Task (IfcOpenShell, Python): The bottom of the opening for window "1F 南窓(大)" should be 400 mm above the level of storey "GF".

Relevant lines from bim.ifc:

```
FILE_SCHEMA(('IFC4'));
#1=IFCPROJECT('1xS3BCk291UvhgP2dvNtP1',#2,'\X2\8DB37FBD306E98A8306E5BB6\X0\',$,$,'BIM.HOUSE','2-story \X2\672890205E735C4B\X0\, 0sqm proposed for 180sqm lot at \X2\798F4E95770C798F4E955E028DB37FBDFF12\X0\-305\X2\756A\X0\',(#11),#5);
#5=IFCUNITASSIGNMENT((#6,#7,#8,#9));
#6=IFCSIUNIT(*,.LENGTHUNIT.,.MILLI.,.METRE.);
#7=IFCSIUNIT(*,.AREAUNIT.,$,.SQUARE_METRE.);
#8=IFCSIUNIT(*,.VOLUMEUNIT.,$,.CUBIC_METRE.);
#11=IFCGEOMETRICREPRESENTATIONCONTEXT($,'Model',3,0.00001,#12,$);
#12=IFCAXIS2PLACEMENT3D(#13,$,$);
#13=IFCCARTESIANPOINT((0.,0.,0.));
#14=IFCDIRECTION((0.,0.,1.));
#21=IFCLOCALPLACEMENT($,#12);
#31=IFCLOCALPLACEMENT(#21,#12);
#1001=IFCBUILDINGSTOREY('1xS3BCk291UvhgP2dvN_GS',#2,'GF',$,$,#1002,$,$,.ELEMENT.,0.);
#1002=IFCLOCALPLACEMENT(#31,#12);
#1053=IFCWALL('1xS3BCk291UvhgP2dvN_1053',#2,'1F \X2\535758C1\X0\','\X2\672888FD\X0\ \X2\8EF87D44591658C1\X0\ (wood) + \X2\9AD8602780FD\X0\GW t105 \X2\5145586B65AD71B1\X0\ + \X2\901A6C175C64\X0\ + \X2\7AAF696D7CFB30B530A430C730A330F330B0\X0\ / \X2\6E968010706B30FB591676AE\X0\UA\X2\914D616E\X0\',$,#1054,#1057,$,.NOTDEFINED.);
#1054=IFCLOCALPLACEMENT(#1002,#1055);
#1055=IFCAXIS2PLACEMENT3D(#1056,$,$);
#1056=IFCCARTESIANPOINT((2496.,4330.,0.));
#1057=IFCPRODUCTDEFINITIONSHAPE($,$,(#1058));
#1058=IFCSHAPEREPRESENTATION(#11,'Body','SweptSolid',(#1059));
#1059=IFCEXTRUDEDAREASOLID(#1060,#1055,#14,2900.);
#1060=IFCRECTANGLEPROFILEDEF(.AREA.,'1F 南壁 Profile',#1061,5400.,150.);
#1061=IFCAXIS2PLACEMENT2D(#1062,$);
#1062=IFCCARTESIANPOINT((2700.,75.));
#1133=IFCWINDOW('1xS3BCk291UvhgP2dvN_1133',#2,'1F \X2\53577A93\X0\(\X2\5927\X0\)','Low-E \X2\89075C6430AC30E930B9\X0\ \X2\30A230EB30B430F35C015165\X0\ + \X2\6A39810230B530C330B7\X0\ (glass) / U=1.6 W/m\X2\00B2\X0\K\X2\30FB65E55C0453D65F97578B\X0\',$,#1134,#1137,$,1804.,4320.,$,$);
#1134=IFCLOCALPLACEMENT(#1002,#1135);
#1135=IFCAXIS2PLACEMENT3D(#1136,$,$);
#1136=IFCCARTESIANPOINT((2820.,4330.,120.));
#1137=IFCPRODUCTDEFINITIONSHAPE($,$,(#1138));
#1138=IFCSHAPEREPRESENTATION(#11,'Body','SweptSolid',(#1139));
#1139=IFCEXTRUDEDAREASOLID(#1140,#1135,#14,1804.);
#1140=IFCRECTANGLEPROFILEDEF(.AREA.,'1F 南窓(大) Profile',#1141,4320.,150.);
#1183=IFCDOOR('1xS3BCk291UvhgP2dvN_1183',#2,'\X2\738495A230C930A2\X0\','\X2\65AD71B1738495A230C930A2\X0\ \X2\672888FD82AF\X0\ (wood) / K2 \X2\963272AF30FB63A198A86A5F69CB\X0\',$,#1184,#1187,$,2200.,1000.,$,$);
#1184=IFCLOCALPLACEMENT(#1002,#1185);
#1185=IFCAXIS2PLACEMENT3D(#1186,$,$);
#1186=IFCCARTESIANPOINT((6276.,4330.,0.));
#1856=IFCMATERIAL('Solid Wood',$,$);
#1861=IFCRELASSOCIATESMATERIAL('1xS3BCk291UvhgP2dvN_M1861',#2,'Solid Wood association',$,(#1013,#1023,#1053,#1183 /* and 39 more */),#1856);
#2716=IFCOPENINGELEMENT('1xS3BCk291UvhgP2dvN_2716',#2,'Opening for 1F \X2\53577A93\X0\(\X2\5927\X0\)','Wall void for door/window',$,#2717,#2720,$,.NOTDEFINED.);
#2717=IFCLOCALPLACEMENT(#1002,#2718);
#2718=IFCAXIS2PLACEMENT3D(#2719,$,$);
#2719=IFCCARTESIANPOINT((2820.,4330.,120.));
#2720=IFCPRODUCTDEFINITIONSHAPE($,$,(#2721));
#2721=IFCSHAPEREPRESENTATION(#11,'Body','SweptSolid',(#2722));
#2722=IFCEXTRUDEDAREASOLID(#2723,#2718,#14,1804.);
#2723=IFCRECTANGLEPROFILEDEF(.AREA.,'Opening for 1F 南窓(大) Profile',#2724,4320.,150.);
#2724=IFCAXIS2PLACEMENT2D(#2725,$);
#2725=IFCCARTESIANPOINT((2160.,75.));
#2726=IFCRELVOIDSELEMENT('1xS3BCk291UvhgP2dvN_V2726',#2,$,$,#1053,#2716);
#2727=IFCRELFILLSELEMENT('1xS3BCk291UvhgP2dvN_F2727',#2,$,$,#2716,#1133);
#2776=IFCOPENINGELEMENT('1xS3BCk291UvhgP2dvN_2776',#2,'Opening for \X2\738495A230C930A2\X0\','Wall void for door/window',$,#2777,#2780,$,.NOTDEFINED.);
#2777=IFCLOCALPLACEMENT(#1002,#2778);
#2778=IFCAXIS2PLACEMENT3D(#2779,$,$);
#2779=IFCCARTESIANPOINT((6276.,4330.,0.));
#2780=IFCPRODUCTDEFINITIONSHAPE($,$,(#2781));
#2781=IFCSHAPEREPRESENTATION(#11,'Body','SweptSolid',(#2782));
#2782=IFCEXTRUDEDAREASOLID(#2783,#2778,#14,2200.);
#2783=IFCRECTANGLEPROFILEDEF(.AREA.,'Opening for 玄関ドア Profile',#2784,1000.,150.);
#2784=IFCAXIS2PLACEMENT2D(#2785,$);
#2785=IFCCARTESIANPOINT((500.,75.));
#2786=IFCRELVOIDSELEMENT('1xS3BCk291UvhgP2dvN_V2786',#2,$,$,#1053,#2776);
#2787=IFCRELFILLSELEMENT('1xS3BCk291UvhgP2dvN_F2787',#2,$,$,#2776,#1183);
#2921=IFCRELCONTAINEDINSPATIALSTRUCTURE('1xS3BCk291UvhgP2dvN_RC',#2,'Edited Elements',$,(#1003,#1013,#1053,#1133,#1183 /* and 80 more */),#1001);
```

```python
import numpy as np
import ifcopenshell
import ifcopenshell.api.geometry
import ifcopenshell.geom
import ifcopenshell.util.element
import ifcopenshell.util.placement
import ifcopenshell.util.shape
import ifcopenshell.util.unit

model = ifcopenshell.open("bim.ifc")
unit_scale = ifcopenshell.util.unit.calculate_unit_scale(model)

window = model.by_guid("1xS3BCk291UvhgP2dvN_1133")
opening = window.FillsVoids[0].RelatingOpeningElement
storey = ifcopenshell.util.element.get_container(window, ifc_class="IfcBuildingStorey")
level = ifcopenshell.util.placement.get_local_placement(storey.ObjectPlacement)[2, 3]

# The opening's origin need not be at the sill, so measure its lowest point.
shape = ifcopenshell.geom.create_shape(ifcopenshell.geom.settings(), opening)
bottom = ifcopenshell.util.shape.get_shape_bottom_elevation(shape, shape.geometry) / unit_scale
dz = level + 400.0 - bottom

shift = np.array([0.0, 0.0, dz])
# The window is not placed relative to its opening, so move both.
for product in (opening, window):
    matrix = ifcopenshell.util.placement.get_local_placement(product.ObjectPlacement)
    matrix[:3, 3] += shift
    ifcopenshell.api.geometry.edit_object_placement(model, product=product, matrix=matrix, is_si=False)

print(f"moved by {dz * unit_scale:+.3f} m")

model.write("bim_updated.ifc")
```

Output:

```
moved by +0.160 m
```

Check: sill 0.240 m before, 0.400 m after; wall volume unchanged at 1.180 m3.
